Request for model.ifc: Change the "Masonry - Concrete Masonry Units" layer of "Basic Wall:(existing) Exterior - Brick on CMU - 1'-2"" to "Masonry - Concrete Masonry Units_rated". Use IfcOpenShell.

First a look at what the model holds.

```python
import ifcopenshell
import ifcopenshell.util.element

model = ifcopenshell.open("model.ifc")
print(model.schema)
for layer_set in model.by_type("IfcMaterialLayerSet"):
    if layer_set.LayerSetName == 'Basic Wall:(existing) Exterior - Brick on CMU - 1\'-2"':
        for layer in layer_set.MaterialLayers:
            print(layer.id(), layer.Material and layer.Material.Name, layer.LayerThickness, sep=" | ")
        print(len(ifcopenshell.util.element.get_elements_by_material(model, layer_set)), "elements and types use it")
print(sorted(m.Name for m in model.by_type("IfcMaterial") if m.Name)[:60])
```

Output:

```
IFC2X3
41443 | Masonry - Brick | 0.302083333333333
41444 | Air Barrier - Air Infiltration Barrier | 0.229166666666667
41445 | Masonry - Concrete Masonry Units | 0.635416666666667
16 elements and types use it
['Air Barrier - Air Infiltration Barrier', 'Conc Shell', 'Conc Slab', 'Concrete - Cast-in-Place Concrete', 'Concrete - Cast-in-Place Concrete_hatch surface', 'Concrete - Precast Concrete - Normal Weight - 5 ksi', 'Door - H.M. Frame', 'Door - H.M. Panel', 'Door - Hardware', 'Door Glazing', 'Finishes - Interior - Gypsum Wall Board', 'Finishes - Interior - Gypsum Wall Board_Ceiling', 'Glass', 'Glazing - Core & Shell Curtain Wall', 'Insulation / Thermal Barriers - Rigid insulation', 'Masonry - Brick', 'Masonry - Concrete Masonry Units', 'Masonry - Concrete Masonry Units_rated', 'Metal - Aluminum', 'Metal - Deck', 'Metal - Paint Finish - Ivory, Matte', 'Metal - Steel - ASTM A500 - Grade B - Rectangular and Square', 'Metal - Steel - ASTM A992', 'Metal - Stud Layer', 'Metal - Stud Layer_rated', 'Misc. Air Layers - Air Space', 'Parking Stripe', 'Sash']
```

```python
import ifcopenshell
import ifcopenshell.api.material

model = ifcopenshell.open("model.ifc")

layer_set = next(s for s in model.by_type("IfcMaterialLayerSet") if s.LayerSetName == 'Basic Wall:(existing) Exterior - Brick on CMU - 1\'-2"')
layer = next(l for l in layer_set.MaterialLayers if l.Material and l.Material.Name == "Masonry - Concrete Masonry Units")
material = next(m for m in model.by_type("IfcMaterial") if m.Name == "Masonry - Concrete Masonry Units_rated")

# Point this one layer at the other material; renaming the old one would change it everywhere.
ifcopenshell.api.material.edit_layer(model, layer=layer, attributes={}, material=material)

print([l.Material.Name if l.Material else None for l in layer_set.MaterialLayers])

model.write("model_edited.ifc")
```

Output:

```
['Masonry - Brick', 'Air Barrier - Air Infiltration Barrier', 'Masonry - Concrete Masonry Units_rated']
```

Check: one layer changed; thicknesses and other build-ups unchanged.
